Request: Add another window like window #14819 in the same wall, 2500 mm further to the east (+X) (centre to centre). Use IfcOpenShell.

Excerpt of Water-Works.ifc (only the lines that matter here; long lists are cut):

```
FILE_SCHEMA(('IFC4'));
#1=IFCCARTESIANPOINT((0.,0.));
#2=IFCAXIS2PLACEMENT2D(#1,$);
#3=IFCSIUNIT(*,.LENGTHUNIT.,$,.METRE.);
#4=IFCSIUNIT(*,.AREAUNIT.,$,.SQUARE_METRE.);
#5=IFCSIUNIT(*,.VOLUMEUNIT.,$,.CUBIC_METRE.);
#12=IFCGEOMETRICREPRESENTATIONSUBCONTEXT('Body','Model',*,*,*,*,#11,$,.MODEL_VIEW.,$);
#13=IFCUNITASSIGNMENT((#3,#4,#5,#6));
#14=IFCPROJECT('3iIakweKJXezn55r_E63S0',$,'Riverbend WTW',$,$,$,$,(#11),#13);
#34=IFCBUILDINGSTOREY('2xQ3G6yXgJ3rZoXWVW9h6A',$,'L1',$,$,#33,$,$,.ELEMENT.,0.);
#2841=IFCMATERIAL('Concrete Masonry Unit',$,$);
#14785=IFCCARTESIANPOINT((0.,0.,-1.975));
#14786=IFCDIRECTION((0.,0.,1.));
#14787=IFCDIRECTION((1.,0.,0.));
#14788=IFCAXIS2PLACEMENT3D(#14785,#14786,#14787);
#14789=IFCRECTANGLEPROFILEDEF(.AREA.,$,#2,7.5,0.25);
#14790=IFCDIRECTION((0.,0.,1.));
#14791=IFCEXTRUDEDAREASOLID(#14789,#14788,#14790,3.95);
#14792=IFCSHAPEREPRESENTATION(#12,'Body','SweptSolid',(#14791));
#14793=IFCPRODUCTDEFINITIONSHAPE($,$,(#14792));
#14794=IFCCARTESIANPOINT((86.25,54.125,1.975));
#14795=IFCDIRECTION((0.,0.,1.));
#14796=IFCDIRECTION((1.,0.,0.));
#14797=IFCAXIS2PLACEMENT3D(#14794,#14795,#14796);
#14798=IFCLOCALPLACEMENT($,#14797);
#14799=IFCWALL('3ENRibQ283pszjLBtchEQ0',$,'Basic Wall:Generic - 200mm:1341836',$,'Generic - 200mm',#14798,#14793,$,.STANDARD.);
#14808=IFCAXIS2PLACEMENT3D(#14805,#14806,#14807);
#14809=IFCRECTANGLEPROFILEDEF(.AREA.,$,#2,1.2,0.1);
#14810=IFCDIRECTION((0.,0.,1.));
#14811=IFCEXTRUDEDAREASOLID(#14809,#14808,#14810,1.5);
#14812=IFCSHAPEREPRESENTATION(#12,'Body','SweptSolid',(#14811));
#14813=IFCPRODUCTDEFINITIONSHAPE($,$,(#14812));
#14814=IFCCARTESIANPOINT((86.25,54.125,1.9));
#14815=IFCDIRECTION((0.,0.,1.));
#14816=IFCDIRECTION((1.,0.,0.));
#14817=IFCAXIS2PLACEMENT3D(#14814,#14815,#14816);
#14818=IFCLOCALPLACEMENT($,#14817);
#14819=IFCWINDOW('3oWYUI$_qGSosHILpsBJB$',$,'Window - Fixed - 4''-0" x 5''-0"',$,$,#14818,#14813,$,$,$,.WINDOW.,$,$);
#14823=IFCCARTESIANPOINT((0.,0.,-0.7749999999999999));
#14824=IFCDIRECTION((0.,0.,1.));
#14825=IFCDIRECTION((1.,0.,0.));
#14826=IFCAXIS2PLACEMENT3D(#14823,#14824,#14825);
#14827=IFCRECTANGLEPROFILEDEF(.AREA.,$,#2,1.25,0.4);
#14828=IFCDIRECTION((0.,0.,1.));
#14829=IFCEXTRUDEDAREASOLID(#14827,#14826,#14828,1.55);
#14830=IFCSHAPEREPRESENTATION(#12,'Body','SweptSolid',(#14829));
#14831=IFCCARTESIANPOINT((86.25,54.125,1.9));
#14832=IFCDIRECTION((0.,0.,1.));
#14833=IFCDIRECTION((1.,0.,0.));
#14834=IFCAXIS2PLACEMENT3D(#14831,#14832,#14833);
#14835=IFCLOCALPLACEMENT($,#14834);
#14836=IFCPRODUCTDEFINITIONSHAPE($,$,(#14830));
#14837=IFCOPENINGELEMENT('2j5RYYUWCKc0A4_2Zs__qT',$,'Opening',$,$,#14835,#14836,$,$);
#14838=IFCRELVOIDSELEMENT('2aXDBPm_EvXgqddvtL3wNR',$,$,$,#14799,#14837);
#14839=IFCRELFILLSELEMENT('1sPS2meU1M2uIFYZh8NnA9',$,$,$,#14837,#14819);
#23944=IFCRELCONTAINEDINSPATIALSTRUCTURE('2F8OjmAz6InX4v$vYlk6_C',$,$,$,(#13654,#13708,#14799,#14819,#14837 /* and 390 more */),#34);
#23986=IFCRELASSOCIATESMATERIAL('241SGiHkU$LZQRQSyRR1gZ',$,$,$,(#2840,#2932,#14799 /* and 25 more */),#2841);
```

```python
import ifcopenshell
import ifcopenshell.api.feature
import ifcopenshell.api.geometry
import ifcopenshell.api.root
import ifcopenshell.geom
import ifcopenshell.util.element
import ifcopenshell.util.placement
import ifcopenshell.util.shape

model = ifcopenshell.open("Water-Works.ifc")
settings = ifcopenshell.geom.settings()


def volume(element):
    """Net volume in cubic metres, openings subtracted."""
    shape = ifcopenshell.geom.create_shape(settings, element)
    return ifcopenshell.util.shape.get_volume(shape.geometry)


window = model.by_guid("3oWYUI$_qGSosHILpsBJB$")
opening = window.FillsVoids[0].RelatingOpeningElement
wall = opening.VoidsElements[0].RelatingBuildingElement
before = volume(wall)
shift = ifcopenshell.util.placement.get_local_placement(wall.ObjectPlacement)[:3, 0] * 2.5

# copy_class copies the void relationship, type, container and properties, but no geometry.
new_opening = ifcopenshell.api.root.copy_class(model, product=opening)
new_opening.Representation = ifcopenshell.util.element.copy_deep(
    model, opening.Representation, exclude=["IfcGeometricRepresentationContext", "IfcRepresentationMap"]
)
new_window = ifcopenshell.api.root.copy_class(model, product=window)
new_window.Representation = ifcopenshell.util.element.copy_deep(
    model, window.Representation, exclude=["IfcGeometricRepresentationContext", "IfcRepresentationMap"]
)
ifcopenshell.api.feature.add_filling(model, opening=new_opening, element=new_window)

for old, new in ((opening, new_opening), (window, new_window)):
    matrix = ifcopenshell.util.placement.get_local_placement(old.ObjectPlacement)
    matrix[:3, 3] += shift
    ifcopenshell.api.geometry.edit_object_placement(model, product=new, matrix=matrix, is_si=False)

after = volume(wall)

print(f"wall volume {before:.3f} -> {after:.3f} m3")

model.write("Water-Works_edited.ifc")
```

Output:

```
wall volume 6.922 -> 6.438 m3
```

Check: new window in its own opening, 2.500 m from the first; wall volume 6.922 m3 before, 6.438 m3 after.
